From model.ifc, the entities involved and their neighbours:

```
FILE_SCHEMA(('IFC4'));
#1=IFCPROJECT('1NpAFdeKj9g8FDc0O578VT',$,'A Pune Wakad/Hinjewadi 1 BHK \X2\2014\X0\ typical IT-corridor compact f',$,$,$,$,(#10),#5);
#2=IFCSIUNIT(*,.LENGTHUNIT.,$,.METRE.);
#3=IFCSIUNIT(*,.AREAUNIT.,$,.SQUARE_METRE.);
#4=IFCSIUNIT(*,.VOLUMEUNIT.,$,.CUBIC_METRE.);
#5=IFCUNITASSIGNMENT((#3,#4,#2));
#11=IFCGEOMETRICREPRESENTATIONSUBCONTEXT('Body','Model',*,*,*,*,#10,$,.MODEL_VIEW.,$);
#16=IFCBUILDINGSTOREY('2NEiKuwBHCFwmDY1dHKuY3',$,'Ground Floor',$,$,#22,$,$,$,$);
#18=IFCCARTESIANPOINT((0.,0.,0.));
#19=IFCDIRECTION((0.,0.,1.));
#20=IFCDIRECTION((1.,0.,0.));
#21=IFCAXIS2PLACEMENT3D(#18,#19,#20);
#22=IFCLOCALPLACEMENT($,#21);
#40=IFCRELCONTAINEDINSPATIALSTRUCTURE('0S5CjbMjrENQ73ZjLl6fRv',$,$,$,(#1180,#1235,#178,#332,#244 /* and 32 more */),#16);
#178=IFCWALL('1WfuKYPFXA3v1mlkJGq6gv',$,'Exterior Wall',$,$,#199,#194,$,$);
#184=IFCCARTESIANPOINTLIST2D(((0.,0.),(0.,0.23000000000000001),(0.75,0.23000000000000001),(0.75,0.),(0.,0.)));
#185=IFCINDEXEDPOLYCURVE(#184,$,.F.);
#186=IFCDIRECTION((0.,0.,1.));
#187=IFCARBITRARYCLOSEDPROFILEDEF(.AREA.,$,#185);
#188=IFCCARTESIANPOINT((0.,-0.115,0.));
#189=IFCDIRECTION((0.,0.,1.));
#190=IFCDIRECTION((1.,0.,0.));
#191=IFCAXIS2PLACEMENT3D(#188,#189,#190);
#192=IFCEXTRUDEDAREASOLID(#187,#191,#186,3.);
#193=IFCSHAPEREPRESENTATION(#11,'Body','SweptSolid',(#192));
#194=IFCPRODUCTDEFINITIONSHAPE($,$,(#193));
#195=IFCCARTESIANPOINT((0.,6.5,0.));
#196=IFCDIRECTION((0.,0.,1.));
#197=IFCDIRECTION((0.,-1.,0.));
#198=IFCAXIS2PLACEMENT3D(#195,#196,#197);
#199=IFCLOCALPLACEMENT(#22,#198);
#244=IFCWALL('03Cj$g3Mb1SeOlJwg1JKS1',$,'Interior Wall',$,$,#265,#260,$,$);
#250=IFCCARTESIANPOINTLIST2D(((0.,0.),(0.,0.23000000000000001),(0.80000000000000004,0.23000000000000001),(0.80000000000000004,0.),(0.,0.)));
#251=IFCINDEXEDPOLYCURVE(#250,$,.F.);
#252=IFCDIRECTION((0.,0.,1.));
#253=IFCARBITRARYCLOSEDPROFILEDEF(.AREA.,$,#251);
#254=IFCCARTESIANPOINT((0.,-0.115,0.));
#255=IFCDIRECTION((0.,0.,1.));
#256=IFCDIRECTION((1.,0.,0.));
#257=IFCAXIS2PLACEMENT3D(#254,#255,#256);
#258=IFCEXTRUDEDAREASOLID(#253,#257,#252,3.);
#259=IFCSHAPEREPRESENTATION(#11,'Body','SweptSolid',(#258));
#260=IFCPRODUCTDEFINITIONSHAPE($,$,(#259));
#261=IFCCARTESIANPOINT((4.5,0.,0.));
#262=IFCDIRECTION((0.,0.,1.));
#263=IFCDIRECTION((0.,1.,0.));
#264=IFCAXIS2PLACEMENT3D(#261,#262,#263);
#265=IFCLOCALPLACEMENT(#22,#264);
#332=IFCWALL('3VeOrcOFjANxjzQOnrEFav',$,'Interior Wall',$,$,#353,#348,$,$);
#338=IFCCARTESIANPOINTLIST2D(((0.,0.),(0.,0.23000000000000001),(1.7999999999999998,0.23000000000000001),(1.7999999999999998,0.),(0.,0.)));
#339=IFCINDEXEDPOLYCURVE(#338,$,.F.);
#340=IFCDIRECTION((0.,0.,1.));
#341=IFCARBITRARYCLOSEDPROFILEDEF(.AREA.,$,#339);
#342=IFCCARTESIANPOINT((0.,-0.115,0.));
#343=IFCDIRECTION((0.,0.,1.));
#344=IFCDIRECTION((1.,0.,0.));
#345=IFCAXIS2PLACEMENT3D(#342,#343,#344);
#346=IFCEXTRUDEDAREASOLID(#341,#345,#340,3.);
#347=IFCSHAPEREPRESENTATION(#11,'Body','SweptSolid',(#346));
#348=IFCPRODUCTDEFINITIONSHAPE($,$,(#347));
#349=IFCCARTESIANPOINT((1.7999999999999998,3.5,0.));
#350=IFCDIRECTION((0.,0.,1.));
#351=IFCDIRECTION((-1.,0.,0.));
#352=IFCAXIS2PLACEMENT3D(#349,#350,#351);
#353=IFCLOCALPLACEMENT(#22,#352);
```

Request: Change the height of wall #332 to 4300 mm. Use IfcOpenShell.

```python
import ifcopenshell
import ifcopenshell.geom
import ifcopenshell.util.representation
import ifcopenshell.util.shape
import ifcopenshell.util.unit

model = ifcopenshell.open("model.ifc")
unit_scale = ifcopenshell.util.unit.calculate_unit_scale(model)
settings = ifcopenshell.geom.settings()


def volume(element):
    """Net volume in cubic metres, openings subtracted."""
    shape = ifcopenshell.geom.create_shape(settings, element)
    return ifcopenshell.util.shape.get_volume(shape.geometry)


wall = model.by_guid("3VeOrcOFjANxjzQOnrEFav")
before = volume(wall)

body = ifcopenshell.util.representation.get_representation(wall, "Model", "Body")
solid = body.Items[0]
old_height = solid.Depth
solid.Depth = 4.3 / unit_scale
after = volume(wall)

print(f"height {old_height:g} -> {solid.Depth:g}, volume {before:.3f} -> {after:.3f} m3")

model.write("model_rev.ifc")
```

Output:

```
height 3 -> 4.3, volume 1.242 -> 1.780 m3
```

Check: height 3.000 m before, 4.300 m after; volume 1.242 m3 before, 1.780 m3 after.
